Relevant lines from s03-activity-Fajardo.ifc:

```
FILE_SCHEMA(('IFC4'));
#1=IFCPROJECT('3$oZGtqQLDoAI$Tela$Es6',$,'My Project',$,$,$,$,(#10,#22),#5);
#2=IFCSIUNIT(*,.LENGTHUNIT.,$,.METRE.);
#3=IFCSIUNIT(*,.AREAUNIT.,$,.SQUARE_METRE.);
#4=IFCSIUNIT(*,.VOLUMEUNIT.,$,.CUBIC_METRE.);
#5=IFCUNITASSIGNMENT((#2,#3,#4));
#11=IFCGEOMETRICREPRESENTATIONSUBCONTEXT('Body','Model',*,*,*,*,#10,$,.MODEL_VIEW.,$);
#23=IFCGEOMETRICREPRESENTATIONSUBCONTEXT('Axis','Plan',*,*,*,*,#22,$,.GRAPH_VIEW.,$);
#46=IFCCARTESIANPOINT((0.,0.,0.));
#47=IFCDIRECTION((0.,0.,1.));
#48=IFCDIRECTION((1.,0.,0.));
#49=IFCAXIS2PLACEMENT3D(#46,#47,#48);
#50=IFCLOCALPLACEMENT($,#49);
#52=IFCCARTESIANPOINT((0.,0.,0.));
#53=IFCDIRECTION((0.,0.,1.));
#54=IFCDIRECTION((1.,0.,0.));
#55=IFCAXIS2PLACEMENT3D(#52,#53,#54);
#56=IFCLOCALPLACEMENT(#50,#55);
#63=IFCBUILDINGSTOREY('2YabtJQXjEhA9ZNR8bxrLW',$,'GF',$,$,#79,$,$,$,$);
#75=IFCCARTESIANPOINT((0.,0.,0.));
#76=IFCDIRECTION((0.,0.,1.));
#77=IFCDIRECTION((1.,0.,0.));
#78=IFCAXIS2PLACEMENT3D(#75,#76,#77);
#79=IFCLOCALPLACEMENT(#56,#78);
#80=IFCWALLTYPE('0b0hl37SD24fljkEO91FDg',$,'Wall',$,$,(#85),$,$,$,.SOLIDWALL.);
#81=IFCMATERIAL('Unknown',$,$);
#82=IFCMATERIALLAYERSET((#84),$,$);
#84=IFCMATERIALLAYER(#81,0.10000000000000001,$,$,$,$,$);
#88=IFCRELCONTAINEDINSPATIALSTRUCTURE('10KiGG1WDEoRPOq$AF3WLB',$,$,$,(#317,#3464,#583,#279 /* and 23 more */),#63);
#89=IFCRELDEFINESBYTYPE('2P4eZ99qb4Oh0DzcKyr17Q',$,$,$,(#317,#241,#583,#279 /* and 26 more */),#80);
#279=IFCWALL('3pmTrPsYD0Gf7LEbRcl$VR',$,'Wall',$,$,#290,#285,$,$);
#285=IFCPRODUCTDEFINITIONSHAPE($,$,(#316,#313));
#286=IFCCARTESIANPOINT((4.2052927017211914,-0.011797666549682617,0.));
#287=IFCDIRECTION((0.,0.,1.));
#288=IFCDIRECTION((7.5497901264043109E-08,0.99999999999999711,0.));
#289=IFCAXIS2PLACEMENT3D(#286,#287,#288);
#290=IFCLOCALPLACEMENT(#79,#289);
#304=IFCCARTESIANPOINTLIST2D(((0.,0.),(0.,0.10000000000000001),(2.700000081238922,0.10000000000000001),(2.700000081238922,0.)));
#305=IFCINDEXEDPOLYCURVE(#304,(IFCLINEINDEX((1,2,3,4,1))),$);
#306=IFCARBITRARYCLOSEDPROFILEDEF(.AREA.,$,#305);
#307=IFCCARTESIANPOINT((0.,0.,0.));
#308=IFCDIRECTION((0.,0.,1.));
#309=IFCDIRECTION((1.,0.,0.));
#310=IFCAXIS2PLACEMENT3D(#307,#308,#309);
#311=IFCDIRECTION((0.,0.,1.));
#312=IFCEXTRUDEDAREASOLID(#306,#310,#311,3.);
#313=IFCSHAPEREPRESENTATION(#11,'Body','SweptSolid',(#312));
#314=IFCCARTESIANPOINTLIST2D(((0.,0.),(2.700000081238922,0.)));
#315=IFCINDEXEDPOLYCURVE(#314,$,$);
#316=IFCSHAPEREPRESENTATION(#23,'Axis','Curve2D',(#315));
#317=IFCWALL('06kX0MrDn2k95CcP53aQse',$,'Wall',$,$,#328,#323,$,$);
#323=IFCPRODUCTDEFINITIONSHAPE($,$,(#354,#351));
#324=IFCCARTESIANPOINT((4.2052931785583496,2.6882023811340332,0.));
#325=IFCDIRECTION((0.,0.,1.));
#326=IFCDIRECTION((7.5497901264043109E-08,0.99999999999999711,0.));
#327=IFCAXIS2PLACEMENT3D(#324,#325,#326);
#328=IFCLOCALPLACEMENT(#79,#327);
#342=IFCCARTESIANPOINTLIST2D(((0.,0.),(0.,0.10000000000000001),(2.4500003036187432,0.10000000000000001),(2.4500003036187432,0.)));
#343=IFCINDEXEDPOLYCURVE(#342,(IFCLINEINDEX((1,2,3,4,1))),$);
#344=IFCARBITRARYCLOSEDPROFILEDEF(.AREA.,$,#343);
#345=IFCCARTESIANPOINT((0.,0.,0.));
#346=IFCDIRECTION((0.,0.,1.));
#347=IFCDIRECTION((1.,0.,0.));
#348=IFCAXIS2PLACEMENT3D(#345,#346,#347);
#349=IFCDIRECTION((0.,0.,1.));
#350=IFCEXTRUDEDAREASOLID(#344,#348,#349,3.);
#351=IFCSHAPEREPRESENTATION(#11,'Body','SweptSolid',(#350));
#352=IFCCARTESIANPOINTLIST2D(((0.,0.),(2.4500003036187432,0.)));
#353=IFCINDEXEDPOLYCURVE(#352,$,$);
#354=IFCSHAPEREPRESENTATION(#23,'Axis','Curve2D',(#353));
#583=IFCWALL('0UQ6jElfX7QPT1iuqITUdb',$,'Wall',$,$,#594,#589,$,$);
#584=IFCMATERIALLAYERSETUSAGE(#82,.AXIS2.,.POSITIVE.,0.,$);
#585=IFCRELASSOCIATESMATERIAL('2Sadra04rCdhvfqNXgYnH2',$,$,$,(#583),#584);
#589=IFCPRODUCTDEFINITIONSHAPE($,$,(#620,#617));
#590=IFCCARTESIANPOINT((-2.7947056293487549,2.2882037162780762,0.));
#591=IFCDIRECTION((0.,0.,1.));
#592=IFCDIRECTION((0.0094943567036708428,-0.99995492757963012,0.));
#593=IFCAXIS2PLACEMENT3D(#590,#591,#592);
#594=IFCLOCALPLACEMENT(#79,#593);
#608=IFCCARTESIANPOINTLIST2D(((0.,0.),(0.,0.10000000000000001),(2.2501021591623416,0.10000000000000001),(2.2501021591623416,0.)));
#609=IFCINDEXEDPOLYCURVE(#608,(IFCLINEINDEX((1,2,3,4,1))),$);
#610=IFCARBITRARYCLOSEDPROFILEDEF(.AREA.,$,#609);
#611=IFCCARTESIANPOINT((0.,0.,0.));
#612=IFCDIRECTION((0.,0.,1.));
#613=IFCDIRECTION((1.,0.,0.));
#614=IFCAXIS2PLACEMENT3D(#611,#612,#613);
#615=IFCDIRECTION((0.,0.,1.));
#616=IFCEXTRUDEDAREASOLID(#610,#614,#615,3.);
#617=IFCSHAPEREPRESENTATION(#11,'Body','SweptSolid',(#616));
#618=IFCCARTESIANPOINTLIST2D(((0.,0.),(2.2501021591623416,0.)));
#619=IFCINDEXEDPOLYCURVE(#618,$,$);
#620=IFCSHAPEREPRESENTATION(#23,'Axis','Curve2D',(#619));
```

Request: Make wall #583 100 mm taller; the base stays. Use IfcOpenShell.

```python
import ifcopenshell
import ifcopenshell.geom
import ifcopenshell.util.representation
import ifcopenshell.util.shape
import ifcopenshell.util.unit

model = ifcopenshell.open("s03-activity-Fajardo.ifc")
unit_scale = ifcopenshell.util.unit.calculate_unit_scale(model)
settings = ifcopenshell.geom.settings()


def volume(element):
    """Net volume in cubic metres, openings subtracted."""
    shape = ifcopenshell.geom.create_shape(settings, element)
    return ifcopenshell.util.shape.get_volume(shape.geometry)


wall = model.by_guid("0UQ6jElfX7QPT1iuqITUdb")
before = volume(wall)

body = ifcopenshell.util.representation.get_representation(wall, "Model", "Body")
solid = body.Items[0]
old_height = solid.Depth
solid.Depth += 0.1 / unit_scale
after = volume(wall)

print(f"height {old_height:g} -> {solid.Depth:g}, volume {before:.3f} -> {after:.3f} m3")

model.write("s03-activity-Fajardo_rev.ifc")
```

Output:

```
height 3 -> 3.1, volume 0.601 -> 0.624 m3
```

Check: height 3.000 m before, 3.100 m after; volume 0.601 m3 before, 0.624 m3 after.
